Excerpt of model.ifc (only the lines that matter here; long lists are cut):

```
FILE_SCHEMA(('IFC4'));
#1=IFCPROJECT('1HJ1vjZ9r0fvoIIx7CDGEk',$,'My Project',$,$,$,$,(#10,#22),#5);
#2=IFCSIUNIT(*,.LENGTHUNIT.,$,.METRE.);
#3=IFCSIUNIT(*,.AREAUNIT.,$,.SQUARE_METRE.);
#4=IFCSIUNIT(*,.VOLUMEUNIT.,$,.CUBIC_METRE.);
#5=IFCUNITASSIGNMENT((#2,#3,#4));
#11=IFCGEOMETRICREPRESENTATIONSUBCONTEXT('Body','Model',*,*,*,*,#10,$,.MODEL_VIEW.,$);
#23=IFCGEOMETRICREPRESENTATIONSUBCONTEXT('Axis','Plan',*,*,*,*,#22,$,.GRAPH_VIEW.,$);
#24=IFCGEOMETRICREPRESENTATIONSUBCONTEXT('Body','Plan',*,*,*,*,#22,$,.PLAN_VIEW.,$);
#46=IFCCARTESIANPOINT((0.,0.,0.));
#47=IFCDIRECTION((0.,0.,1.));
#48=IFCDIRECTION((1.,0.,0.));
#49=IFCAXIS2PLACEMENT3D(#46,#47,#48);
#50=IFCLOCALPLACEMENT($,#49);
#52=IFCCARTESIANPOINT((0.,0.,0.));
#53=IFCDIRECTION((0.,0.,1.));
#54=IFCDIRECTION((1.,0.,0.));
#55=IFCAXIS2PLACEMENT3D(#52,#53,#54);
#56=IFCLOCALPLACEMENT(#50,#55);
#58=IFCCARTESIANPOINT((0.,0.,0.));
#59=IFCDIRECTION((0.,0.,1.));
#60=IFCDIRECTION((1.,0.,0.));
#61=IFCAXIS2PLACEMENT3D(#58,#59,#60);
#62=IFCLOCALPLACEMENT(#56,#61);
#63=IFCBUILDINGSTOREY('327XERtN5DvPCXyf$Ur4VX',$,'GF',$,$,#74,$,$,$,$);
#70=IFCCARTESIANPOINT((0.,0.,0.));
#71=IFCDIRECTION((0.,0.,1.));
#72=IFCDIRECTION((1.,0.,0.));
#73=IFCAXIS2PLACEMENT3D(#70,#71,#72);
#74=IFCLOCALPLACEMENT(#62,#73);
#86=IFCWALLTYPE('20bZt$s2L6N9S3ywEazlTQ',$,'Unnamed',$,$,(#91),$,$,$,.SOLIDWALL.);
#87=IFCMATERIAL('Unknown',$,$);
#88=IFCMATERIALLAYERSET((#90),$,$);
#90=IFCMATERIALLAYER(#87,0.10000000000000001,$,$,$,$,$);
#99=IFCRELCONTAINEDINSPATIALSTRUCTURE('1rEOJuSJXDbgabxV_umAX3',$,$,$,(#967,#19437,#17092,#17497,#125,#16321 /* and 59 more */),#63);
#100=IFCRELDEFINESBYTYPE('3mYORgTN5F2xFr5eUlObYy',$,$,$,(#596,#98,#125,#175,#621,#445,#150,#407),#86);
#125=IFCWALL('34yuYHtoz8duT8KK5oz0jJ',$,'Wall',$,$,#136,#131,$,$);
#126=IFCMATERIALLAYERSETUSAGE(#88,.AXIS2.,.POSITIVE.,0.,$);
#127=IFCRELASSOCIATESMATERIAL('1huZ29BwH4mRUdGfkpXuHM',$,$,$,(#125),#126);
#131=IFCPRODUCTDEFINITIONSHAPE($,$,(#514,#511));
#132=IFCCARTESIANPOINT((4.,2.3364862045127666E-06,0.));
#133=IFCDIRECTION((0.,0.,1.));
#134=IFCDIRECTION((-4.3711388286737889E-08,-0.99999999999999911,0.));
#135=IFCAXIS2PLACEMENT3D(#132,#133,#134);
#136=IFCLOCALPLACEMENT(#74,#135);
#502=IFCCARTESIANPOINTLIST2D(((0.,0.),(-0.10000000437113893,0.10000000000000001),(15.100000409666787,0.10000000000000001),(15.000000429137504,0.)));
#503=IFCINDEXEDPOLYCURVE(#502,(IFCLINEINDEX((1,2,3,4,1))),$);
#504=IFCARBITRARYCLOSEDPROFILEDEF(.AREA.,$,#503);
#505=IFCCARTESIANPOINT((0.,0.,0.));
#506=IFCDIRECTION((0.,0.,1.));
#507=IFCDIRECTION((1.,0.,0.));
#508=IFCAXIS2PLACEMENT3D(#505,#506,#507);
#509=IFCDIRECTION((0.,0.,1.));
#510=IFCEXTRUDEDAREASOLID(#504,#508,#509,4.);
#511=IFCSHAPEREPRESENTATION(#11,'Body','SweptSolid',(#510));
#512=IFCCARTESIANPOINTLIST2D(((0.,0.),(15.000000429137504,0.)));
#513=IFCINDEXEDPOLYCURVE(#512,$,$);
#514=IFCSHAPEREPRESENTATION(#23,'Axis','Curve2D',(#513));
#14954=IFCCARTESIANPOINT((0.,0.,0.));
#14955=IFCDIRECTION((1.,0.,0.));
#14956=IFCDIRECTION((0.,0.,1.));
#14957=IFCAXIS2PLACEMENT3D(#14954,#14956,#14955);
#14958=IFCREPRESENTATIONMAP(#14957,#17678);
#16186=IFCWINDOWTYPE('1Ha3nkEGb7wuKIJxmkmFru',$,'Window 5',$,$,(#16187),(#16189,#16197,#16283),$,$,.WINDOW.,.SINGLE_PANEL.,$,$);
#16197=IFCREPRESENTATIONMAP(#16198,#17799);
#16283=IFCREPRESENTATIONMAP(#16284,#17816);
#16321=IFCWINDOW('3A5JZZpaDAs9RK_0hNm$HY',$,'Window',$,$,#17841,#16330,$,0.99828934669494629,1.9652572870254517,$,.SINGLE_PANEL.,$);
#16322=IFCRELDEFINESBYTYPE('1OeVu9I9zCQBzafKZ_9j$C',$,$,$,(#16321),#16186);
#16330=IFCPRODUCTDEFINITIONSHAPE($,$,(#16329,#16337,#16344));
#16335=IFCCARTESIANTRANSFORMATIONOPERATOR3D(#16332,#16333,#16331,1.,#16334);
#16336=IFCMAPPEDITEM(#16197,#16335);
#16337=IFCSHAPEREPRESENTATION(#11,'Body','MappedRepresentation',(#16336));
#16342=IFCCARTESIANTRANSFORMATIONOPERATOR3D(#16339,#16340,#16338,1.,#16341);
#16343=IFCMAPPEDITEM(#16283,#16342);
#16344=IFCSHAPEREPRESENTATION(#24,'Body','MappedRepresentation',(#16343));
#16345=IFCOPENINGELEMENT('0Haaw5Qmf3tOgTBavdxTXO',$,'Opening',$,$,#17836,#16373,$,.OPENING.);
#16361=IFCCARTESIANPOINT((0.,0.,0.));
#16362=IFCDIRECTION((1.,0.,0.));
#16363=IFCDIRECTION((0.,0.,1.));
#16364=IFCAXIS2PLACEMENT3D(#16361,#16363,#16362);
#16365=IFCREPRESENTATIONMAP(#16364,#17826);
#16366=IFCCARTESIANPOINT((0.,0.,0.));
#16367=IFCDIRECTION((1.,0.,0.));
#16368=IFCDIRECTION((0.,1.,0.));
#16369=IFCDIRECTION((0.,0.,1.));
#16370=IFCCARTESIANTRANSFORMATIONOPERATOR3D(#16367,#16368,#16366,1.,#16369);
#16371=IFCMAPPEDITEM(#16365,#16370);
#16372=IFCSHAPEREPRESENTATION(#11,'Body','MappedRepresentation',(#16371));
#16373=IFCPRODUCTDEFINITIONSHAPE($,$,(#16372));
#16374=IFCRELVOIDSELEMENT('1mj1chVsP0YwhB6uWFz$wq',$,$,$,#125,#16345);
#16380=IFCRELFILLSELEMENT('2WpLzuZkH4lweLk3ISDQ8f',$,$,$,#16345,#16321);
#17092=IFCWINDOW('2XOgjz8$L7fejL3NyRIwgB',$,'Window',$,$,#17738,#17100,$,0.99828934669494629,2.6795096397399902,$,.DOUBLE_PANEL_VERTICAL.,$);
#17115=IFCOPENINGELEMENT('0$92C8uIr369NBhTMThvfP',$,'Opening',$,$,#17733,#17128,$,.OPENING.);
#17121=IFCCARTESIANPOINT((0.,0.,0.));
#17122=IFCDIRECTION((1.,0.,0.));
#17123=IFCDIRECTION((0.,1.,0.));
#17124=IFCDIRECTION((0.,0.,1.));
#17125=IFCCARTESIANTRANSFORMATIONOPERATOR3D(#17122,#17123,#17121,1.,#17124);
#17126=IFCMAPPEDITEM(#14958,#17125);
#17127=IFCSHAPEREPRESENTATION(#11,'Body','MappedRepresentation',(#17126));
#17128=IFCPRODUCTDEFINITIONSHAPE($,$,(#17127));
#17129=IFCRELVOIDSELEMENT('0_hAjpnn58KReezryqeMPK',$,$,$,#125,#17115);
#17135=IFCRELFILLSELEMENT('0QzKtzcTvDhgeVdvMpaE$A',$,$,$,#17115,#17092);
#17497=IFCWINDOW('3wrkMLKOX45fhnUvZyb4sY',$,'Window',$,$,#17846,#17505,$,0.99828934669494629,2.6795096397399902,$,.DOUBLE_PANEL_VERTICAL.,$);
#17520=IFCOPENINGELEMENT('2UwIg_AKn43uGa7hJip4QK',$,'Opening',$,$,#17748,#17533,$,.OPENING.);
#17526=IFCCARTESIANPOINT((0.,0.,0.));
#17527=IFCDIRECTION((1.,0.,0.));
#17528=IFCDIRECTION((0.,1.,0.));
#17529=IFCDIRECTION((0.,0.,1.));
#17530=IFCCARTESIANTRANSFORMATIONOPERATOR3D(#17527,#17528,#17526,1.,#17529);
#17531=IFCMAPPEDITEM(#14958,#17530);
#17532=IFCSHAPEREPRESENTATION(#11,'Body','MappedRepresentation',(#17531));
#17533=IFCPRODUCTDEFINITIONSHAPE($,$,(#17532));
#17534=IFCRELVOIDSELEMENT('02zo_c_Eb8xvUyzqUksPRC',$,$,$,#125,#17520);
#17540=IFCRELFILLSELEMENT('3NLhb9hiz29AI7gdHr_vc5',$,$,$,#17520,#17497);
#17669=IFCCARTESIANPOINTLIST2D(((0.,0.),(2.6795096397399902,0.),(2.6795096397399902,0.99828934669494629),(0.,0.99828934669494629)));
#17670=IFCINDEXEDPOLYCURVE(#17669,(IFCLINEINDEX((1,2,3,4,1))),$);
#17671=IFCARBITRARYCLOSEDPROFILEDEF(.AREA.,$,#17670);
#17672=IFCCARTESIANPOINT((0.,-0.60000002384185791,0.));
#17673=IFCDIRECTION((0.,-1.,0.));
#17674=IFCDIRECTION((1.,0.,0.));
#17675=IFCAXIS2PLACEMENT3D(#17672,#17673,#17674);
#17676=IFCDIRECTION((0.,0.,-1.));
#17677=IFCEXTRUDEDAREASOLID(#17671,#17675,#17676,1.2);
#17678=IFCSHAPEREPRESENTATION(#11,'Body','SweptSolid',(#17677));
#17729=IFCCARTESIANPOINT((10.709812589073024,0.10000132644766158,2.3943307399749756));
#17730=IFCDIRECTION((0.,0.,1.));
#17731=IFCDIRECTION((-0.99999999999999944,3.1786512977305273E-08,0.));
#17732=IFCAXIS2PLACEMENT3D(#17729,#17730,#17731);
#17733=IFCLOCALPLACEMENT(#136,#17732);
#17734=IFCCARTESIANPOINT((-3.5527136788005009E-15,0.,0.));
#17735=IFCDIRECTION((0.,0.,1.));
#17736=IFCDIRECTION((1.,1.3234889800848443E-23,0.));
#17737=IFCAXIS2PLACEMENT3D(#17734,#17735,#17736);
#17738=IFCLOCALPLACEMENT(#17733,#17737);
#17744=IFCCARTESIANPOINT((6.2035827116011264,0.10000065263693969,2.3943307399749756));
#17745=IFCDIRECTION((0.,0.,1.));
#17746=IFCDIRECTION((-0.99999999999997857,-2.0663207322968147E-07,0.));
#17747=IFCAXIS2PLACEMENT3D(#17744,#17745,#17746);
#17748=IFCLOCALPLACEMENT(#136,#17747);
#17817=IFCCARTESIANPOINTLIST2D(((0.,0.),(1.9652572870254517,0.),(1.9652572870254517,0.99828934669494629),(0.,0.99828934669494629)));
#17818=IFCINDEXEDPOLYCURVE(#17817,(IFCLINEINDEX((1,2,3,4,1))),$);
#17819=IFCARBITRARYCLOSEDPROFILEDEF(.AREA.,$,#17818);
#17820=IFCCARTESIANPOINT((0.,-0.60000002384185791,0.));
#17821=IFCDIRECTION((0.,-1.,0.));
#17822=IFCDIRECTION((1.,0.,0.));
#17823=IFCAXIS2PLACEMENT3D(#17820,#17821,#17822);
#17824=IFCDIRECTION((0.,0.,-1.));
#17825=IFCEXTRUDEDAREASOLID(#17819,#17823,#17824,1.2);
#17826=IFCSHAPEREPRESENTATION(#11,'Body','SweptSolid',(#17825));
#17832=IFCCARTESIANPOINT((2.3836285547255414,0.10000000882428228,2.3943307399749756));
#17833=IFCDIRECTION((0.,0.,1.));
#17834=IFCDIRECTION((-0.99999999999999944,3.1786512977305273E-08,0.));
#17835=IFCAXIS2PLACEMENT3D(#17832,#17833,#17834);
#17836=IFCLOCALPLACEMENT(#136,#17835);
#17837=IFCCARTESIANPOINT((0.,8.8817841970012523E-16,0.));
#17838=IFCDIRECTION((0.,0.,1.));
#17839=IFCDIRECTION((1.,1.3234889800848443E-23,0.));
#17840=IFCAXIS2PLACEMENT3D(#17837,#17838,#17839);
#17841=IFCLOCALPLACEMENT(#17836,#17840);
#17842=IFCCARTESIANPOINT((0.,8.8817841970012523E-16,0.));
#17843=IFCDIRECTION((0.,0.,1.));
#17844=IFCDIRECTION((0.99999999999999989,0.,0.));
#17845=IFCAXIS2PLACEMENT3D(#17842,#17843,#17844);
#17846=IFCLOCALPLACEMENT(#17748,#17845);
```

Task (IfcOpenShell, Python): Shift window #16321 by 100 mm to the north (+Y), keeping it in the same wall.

```python
import ifcopenshell
import ifcopenshell.api.geometry
import ifcopenshell.util.placement
import ifcopenshell.util.unit

model = ifcopenshell.open("model.ifc")
unit_scale = ifcopenshell.util.unit.calculate_unit_scale(model)

window = model.by_guid("3A5JZZpaDAs9RK_0hNm$HY")
opening = window.FillsVoids[0].RelatingOpeningElement
wall = opening.VoidsElements[0].RelatingBuildingElement

wall_matrix = ifcopenshell.util.placement.get_local_placement(wall.ObjectPlacement)
shift = wall_matrix[:3, 0] * -0.1 / unit_scale
before = ifcopenshell.util.placement.get_local_placement(window.ObjectPlacement)[:3, 3].copy()

# The window is placed relative to its opening, so it follows when the opening moves.
matrix = ifcopenshell.util.placement.get_local_placement(opening.ObjectPlacement)
matrix[:3, 3] += shift
ifcopenshell.api.geometry.edit_object_placement(
    model, product=opening, matrix=matrix, is_si=False, should_transform_children=True
)

after = ifcopenshell.util.placement.get_local_placement(window.ObjectPlacement)[:3, 3]
print("window moved by", (after - before).round(3) + 0.0)

model.write("model_v2.ifc")
```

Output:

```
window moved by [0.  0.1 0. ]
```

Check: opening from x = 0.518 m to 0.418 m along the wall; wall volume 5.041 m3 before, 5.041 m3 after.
